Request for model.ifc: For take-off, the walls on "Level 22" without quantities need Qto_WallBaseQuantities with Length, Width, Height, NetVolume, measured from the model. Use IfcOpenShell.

First a look at what the model holds.

```python
import ifcopenshell
import ifcopenshell.util.element
import ifcopenshell.util.unit

model = ifcopenshell.open("model.ifc")
print(model.schema)
for unit_type in ("LENGTHUNIT", "AREAUNIT", "VOLUMEUNIT"):
    print(unit_type, ifcopenshell.util.unit.calculate_unit_scale(model, unit_type))
storey = next(s for s in model.by_type("IfcBuildingStorey") if s.Name == "Level 22")
walls = [e for e in ifcopenshell.util.element.get_decomposition(storey) if e.is_a("IfcWall")]
for e in sorted(walls, key=lambda e: e.id()):
    print(e.id(), e.is_a(), e.Name, list(ifcopenshell.util.element.get_psets(e, qtos_only=True)), sep=" | ")
```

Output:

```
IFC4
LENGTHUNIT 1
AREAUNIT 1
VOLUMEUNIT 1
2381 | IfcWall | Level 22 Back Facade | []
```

```python
import ifcopenshell
import ifcopenshell.api.pset
import ifcopenshell.geom
import ifcopenshell.util.element
import ifcopenshell.util.shape
import ifcopenshell.util.unit

model = ifcopenshell.open("model.ifc")
unit_scale = ifcopenshell.util.unit.calculate_unit_scale(model)
volume_scale = ifcopenshell.util.unit.calculate_unit_scale(model, "VOLUMEUNIT")
settings = ifcopenshell.geom.settings()

storey = next(s for s in model.by_type("IfcBuildingStorey") if s.Name == "Level 22")
walls = [e for e in ifcopenshell.util.element.get_decomposition(storey) if e.is_a("IfcWall")]

for e in sorted(walls, key=lambda e: e.id()):
    if ifcopenshell.util.element.get_psets(e, qtos_only=True, should_inherit=False):
        continue
    # Geometry comes back in metres, in the element's own axes.
    shape = ifcopenshell.geom.create_shape(settings, e)
    values = {
        "Length": ifcopenshell.util.shape.get_x(shape.geometry) / unit_scale,
        "Width": ifcopenshell.util.shape.get_y(shape.geometry) / unit_scale,
        "Height": ifcopenshell.util.shape.get_z(shape.geometry) / unit_scale,
        "NetVolume": ifcopenshell.util.shape.get_volume(shape.geometry) / volume_scale,
    }
    qto = ifcopenshell.api.pset.add_qto(model, product=e, name="Qto_WallBaseQuantities")
    ifcopenshell.api.pset.edit_qto(model, qto=qto, properties=values)
    print(e.id(), {k: round(v, 3) for k, v in values.items()})

model.write("model_rev.ifc")
```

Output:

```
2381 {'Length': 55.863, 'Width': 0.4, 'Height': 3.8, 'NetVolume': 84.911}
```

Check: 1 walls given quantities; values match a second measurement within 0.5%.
